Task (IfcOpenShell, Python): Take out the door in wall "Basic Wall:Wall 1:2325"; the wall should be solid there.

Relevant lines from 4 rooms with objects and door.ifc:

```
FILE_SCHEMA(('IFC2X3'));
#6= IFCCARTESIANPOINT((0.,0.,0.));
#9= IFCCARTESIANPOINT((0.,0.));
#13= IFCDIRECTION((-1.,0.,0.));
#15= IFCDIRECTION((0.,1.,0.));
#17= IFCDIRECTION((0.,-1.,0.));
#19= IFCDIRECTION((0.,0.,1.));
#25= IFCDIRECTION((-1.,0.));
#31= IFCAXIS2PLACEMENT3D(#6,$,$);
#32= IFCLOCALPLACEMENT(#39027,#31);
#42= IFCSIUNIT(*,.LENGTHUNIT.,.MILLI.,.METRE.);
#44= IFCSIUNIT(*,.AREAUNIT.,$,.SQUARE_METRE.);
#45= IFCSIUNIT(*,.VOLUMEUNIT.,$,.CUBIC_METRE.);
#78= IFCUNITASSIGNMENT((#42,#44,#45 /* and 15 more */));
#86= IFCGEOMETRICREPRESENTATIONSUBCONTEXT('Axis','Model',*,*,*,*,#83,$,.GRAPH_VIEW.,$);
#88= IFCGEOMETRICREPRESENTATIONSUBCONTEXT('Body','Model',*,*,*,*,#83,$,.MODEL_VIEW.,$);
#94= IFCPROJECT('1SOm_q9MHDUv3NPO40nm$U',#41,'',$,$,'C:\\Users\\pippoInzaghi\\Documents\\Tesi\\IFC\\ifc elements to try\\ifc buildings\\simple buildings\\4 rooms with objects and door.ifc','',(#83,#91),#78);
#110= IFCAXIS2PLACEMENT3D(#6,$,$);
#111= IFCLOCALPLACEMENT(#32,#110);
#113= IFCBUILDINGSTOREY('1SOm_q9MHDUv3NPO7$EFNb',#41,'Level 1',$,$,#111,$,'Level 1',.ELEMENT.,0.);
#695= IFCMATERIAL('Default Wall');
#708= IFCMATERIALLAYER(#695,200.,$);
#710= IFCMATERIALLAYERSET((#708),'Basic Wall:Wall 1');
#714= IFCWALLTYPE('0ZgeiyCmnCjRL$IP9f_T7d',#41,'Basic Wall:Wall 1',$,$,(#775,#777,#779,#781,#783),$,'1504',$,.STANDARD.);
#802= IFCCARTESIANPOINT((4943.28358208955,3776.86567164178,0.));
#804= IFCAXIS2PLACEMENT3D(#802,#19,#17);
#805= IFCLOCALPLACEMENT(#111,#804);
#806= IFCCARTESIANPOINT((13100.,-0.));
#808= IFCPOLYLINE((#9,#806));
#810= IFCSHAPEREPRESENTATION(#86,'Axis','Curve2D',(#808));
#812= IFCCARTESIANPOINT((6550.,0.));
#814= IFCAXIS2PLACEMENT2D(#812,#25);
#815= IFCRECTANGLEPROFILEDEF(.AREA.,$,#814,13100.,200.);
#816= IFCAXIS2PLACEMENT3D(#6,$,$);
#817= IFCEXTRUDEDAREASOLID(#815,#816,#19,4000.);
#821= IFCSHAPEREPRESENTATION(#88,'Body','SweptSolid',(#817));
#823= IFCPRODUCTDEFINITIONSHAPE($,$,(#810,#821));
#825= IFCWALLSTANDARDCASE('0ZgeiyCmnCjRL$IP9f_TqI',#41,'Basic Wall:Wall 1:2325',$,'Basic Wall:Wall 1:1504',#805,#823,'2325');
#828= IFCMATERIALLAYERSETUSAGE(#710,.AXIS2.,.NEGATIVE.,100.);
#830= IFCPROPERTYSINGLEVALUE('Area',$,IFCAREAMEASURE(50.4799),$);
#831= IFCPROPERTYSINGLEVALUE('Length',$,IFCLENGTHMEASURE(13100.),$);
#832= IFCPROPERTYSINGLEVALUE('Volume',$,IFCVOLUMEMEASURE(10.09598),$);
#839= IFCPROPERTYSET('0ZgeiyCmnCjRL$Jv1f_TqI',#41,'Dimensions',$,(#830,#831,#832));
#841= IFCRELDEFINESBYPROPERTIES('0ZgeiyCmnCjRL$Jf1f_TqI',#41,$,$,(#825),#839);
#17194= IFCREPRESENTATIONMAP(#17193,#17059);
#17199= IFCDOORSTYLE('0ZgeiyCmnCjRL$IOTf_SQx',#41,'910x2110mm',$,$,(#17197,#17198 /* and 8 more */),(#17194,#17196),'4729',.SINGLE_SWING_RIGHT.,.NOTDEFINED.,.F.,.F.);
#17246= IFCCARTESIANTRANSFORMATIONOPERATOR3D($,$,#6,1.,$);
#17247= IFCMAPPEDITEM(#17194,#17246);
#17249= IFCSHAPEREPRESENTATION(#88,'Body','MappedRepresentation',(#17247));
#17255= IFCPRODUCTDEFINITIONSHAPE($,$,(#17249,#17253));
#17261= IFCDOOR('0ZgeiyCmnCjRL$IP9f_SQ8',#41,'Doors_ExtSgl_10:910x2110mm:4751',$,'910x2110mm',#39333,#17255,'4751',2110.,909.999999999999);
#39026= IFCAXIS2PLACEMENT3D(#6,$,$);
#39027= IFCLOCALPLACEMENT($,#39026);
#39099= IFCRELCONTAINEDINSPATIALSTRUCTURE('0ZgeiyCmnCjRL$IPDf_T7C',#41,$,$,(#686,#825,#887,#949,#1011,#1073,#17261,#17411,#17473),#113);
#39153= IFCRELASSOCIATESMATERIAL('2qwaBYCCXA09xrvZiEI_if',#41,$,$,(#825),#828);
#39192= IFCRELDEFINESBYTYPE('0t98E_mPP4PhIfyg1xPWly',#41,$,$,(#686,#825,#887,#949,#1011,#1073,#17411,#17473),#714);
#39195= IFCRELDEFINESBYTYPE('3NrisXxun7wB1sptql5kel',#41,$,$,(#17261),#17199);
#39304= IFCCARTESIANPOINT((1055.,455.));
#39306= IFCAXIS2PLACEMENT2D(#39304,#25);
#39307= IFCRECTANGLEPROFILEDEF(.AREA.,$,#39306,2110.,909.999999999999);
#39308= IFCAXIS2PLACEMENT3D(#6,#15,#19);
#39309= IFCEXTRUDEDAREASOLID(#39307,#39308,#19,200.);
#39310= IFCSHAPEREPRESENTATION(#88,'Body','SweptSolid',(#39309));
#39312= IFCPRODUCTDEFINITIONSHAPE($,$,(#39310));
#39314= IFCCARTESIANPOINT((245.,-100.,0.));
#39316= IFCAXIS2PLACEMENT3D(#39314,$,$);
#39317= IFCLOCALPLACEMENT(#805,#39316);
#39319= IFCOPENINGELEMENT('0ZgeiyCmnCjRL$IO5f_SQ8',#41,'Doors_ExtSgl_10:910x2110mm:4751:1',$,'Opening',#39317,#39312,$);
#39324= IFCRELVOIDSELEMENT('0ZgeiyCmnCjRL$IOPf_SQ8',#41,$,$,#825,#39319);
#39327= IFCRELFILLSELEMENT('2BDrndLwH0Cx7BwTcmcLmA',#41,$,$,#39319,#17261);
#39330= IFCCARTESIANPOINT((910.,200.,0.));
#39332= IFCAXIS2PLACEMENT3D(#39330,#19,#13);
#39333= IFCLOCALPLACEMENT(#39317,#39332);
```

```python
import ifcopenshell
import ifcopenshell.api.feature
import ifcopenshell.api.pset
import ifcopenshell.api.root
import ifcopenshell.geom
import ifcopenshell.util.element
import ifcopenshell.util.shape
import ifcopenshell.util.unit

model = ifcopenshell.open("4 rooms with objects and door.ifc")
area_scale = ifcopenshell.util.unit.calculate_unit_scale(model, "AREAUNIT")
volume_scale = ifcopenshell.util.unit.calculate_unit_scale(model, "VOLUMEUNIT")
settings = ifcopenshell.geom.settings()


def volume(element):
    """Net volume in cubic metres, openings subtracted."""
    shape = ifcopenshell.geom.create_shape(settings, element)
    return ifcopenshell.util.shape.get_volume(shape.geometry)


door = model.by_id(17261)
opening = door.FillsVoids[0].RelatingOpeningElement
wall = opening.VoidsElements[0].RelatingBuildingElement
before = volume(wall)

ifcopenshell.api.root.remove_product(model, product=door)
ifcopenshell.api.feature.remove_feature(model, feature=opening)

after = volume(wall)
thickness = 0.2  # wall thickness in metres

# Update the wall's stored quantities.
pset = model.by_id(ifcopenshell.util.element.get_pset(wall, "Dimensions", should_inherit=False)["id"])
ifcopenshell.api.pset.edit_pset(model, pset=pset, properties={
    "Area": model.create_entity("IfcAreaMeasure", after / thickness / area_scale),
    "Volume": model.create_entity("IfcVolumeMeasure", after / volume_scale),
})

print(f"wall volume {before:.3f} -> {after:.3f} m3")

model.write("4 rooms with objects and door_v2.ifc")
```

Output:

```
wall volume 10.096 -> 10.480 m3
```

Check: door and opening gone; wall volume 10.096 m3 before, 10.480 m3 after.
